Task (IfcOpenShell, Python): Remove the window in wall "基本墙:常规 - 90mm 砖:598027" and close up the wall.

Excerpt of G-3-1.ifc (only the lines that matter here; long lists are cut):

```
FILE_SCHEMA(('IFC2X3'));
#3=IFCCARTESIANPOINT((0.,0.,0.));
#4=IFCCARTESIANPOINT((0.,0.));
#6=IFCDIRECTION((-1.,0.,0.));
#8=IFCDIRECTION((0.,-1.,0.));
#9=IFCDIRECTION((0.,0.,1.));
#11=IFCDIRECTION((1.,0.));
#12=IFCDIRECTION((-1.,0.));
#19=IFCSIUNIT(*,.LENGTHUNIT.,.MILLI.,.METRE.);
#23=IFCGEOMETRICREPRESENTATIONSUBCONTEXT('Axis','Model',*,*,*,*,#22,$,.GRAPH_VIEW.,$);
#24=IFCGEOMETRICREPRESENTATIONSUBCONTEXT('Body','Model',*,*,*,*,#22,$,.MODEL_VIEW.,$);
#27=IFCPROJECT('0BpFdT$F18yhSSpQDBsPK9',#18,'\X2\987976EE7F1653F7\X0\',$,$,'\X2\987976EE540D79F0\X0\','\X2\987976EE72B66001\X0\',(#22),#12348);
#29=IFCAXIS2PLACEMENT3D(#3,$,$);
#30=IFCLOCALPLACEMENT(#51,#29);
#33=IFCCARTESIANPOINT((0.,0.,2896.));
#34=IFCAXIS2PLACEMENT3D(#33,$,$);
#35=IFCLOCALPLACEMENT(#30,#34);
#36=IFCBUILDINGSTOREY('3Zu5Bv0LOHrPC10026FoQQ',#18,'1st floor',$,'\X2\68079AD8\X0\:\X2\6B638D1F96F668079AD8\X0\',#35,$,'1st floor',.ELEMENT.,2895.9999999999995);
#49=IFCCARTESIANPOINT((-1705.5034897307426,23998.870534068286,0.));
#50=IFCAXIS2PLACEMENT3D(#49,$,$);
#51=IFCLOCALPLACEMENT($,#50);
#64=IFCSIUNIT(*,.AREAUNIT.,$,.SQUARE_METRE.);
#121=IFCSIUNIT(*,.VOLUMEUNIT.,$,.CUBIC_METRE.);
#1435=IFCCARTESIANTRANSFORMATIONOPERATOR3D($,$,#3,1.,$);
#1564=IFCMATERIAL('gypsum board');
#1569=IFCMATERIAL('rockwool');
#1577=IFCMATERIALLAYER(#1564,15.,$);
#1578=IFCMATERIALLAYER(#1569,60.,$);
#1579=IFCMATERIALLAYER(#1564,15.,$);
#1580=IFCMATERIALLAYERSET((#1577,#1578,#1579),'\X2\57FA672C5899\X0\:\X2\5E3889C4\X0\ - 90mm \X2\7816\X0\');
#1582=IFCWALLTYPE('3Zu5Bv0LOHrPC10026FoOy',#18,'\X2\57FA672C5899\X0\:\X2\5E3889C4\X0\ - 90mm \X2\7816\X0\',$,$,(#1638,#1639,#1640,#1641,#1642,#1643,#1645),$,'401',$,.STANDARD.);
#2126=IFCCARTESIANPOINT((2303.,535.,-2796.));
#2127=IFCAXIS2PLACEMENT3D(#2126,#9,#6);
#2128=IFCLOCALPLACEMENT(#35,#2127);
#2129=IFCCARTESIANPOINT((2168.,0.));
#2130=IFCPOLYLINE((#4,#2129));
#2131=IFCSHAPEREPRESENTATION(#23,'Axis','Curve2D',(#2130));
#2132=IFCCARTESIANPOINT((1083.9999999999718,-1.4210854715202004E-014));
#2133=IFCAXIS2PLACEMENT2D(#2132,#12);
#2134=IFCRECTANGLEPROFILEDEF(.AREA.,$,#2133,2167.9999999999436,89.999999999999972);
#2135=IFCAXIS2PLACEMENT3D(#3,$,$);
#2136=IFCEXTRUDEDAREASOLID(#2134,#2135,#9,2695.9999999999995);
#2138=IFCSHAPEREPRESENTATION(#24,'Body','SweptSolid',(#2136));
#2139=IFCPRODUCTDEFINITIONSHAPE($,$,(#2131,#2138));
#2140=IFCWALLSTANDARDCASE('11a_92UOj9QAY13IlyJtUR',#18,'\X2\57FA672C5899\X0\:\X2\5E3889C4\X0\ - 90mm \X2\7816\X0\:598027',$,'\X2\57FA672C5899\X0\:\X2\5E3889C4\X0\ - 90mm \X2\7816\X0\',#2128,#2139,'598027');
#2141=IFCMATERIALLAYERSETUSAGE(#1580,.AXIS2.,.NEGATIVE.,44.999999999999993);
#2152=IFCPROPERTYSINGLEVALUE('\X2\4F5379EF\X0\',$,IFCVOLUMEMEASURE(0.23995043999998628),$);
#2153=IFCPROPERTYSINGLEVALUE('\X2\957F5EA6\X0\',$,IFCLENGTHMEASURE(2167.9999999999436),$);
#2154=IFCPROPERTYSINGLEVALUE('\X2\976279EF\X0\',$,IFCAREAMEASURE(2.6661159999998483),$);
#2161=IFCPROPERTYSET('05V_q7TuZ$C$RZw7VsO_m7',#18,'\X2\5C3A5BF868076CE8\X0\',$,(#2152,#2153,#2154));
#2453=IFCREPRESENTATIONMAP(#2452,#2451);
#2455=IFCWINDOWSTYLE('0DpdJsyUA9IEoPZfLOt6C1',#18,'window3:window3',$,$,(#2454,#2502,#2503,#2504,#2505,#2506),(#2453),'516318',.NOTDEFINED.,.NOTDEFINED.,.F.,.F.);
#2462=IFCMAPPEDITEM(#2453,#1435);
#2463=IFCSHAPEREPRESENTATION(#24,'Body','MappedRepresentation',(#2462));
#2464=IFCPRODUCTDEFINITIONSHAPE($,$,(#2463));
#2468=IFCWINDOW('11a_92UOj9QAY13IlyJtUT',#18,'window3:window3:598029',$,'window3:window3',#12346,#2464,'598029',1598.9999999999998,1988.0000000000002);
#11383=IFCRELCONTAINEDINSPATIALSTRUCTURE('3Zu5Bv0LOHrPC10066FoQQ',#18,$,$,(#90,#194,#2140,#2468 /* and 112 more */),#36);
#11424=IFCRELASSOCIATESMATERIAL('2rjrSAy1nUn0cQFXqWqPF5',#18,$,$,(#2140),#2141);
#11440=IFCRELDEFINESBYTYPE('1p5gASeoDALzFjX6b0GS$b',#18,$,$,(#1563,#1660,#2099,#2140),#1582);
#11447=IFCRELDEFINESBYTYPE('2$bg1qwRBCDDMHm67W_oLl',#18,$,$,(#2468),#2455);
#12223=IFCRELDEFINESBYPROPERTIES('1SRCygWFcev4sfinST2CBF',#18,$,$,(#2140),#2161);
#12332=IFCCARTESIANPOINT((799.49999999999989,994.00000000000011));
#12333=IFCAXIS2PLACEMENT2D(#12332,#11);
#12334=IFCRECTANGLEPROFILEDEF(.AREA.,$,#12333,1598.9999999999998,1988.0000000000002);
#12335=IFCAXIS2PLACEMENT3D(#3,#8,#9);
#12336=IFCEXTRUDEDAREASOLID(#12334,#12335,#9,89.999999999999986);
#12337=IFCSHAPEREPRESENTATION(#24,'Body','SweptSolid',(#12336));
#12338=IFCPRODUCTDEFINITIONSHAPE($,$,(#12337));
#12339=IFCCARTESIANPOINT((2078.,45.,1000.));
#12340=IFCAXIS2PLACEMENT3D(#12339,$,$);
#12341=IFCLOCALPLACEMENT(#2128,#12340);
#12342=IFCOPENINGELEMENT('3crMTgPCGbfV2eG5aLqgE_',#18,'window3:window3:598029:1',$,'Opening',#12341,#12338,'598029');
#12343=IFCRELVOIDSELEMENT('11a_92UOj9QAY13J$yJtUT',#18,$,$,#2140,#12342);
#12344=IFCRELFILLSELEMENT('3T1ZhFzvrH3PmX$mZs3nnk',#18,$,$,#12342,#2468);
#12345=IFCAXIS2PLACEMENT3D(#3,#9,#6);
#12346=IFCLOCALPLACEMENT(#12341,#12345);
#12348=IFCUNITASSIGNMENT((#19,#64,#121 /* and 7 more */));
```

```python
import ifcopenshell
import ifcopenshell.api.feature
import ifcopenshell.api.pset
import ifcopenshell.api.root
import ifcopenshell.geom
import ifcopenshell.util.element
import ifcopenshell.util.shape
import ifcopenshell.util.unit

model = ifcopenshell.open("G-3-1.ifc")
area_scale = ifcopenshell.util.unit.calculate_unit_scale(model, "AREAUNIT")
volume_scale = ifcopenshell.util.unit.calculate_unit_scale(model, "VOLUMEUNIT")
settings = ifcopenshell.geom.settings()


def volume(element):
    """Net volume in cubic metres, openings subtracted."""
    shape = ifcopenshell.geom.create_shape(settings, element)
    return ifcopenshell.util.shape.get_volume(shape.geometry)


window = model.by_id(2468)
opening = window.FillsVoids[0].RelatingOpeningElement
wall = opening.VoidsElements[0].RelatingBuildingElement
before = volume(wall)

ifcopenshell.api.root.remove_product(model, product=window)
ifcopenshell.api.feature.remove_feature(model, feature=opening)

after = volume(wall)
thickness = 0.09  # wall thickness in metres

# Update the wall's stored quantities.
pset = model.by_id(ifcopenshell.util.element.get_pset(wall, "尺寸标注", should_inherit=False)["id"])
ifcopenshell.api.pset.edit_pset(model, pset=pset, properties={
    "体积": model.create_entity("IfcVolumeMeasure", after / volume_scale),
    "面积": model.create_entity("IfcAreaMeasure", after / thickness / area_scale),
})

print(f"wall volume {before:.3f} -> {after:.3f} m3")

model.write("G-3-1_rev.ifc")
```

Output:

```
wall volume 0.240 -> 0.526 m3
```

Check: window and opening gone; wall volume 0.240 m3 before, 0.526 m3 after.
